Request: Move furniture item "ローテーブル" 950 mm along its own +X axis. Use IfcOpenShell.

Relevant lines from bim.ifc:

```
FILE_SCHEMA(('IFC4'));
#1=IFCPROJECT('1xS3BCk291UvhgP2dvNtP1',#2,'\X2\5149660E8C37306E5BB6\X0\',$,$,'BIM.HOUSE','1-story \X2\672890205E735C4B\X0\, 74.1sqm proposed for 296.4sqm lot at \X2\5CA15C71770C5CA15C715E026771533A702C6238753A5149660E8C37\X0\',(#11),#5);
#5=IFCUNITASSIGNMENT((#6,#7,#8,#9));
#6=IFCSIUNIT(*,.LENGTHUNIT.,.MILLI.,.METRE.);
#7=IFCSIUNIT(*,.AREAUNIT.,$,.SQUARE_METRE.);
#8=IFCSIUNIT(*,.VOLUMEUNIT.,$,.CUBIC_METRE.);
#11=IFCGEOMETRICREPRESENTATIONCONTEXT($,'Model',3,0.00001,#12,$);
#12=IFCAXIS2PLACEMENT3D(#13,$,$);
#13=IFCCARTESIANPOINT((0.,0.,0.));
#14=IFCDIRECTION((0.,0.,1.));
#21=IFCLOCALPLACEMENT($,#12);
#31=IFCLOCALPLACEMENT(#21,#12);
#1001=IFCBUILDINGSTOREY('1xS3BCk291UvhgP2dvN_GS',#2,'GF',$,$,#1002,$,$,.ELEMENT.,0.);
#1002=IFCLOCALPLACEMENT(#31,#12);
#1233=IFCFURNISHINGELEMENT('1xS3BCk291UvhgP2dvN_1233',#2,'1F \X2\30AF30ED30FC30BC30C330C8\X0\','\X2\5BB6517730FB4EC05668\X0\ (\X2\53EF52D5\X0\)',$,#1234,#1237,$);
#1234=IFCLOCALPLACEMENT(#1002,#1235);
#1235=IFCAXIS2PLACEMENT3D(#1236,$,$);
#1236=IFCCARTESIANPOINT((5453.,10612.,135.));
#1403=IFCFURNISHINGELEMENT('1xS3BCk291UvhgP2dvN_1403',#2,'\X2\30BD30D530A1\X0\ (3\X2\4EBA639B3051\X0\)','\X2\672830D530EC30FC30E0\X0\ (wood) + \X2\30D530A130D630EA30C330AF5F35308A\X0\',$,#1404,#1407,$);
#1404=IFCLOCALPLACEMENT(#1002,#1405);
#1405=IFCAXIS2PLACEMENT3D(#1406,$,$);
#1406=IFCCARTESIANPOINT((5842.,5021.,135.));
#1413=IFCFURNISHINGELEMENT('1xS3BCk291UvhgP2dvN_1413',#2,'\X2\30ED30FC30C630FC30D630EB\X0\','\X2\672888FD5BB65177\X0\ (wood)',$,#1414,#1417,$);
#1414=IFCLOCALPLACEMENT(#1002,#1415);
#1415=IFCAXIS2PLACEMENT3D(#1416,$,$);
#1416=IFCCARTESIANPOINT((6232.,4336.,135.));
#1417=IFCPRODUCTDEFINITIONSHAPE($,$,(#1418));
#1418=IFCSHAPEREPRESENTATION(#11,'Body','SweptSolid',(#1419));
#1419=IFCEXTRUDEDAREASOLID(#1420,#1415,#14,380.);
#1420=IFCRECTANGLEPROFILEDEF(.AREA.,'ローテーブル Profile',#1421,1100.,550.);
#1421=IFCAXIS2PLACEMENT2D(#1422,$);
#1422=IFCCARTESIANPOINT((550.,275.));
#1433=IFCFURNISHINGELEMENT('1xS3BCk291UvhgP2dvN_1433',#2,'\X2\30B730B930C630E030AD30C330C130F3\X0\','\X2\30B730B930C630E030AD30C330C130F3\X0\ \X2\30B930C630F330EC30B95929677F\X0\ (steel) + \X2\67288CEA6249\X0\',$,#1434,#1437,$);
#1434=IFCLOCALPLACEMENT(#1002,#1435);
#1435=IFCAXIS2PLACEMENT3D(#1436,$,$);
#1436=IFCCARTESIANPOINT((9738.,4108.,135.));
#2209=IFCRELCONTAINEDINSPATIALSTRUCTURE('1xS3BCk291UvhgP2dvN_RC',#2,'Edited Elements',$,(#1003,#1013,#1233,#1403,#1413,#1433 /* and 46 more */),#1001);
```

```python
import ifcopenshell
import ifcopenshell.api.geometry
import ifcopenshell.util.placement

model = ifcopenshell.open("bim.ifc")

item = model.by_guid("1xS3BCk291UvhgP2dvN_1413")
matrix = ifcopenshell.util.placement.get_local_placement(item.ObjectPlacement)
matrix[:3, 3] += matrix[:3, 0] * 950.0
ifcopenshell.api.geometry.edit_object_placement(model, product=item, matrix=matrix, is_si=False)

print(ifcopenshell.util.placement.get_local_placement(item.ObjectPlacement).round(3) + 0.0)

model.write("bim_rev.ifc")
```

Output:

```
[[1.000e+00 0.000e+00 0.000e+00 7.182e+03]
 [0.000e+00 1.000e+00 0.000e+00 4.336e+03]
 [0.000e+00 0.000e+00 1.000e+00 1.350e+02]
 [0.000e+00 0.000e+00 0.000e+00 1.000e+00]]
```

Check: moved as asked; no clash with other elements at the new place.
